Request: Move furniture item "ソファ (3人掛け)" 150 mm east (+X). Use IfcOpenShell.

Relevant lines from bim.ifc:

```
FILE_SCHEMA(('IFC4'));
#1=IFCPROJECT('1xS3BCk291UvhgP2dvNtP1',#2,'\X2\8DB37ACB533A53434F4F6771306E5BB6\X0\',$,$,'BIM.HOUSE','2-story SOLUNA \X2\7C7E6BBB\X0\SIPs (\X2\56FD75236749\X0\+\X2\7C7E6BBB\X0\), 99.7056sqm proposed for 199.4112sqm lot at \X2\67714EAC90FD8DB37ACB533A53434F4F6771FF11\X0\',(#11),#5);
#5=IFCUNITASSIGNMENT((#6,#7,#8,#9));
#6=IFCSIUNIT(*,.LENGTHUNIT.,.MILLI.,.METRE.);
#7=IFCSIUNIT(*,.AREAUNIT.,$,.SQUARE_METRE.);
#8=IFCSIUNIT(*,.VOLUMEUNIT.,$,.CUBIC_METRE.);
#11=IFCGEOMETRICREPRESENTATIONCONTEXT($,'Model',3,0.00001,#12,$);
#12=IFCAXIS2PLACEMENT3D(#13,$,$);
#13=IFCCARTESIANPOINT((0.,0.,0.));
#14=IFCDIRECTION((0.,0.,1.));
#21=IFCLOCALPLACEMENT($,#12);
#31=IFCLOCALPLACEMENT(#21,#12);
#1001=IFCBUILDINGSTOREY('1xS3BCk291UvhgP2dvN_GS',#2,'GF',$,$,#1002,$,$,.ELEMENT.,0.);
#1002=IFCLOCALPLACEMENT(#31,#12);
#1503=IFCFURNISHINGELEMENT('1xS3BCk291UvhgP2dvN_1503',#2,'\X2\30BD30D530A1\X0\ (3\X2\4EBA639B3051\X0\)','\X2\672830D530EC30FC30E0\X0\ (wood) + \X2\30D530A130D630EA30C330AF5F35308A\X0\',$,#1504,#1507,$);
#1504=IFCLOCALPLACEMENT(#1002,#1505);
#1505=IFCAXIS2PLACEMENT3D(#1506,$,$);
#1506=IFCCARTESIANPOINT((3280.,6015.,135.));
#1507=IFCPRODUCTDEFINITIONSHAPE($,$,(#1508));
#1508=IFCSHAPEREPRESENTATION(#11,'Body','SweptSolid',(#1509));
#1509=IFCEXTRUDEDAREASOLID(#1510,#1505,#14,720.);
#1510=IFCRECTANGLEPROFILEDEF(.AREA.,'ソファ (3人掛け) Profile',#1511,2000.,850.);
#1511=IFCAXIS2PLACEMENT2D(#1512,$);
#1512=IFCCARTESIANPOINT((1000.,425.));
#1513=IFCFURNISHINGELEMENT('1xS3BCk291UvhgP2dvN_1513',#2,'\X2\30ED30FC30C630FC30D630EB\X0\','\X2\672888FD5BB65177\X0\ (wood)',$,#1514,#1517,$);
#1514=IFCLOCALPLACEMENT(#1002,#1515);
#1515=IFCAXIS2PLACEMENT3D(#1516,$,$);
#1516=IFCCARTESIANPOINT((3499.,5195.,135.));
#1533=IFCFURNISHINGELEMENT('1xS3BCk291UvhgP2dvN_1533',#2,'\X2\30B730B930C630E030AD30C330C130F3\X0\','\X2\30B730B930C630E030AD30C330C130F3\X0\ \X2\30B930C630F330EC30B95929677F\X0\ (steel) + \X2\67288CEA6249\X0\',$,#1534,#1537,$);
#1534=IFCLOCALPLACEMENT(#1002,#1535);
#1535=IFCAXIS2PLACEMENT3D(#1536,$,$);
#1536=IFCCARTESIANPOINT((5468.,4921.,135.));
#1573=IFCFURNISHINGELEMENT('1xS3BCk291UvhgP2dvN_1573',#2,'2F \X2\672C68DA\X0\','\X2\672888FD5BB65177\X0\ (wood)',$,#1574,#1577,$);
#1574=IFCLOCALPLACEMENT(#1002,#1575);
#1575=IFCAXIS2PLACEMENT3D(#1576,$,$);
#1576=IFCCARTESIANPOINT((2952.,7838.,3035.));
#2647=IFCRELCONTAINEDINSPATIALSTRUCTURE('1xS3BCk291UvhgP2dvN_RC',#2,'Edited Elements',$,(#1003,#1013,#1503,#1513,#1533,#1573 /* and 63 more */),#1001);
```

```python
import ifcopenshell
import ifcopenshell.api.geometry
import ifcopenshell.util.placement
import ifcopenshell.util.unit

model = ifcopenshell.open("bim.ifc")
unit_scale = ifcopenshell.util.unit.calculate_unit_scale(model)

item = model.by_id(1503)
matrix = ifcopenshell.util.placement.get_local_placement(item.ObjectPlacement)
matrix[0, 3] += 0.15 / unit_scale
ifcopenshell.api.geometry.edit_object_placement(model, product=item, matrix=matrix, is_si=False)

print(ifcopenshell.util.placement.get_local_placement(item.ObjectPlacement).round(3) + 0.0)

model.write("bim_rev.ifc")
```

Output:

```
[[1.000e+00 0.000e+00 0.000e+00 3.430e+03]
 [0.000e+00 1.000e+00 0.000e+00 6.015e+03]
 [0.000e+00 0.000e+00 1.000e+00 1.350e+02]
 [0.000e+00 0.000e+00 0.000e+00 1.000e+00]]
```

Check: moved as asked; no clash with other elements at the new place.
